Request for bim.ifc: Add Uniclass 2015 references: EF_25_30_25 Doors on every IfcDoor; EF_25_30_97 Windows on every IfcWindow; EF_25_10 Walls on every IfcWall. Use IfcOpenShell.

First a look at what the model holds.

```python
import ifcopenshell

model = ifcopenshell.open("bim.ifc")
print(model.schema)
print("classifications:", [c.Name for c in model.by_type("IfcClassification")])
for ifc_class in ("IfcDoor", "IfcRoof", "IfcStair", "IfcWall", "IfcWindow"):
    print(ifc_class, len(model.by_type(ifc_class)))
```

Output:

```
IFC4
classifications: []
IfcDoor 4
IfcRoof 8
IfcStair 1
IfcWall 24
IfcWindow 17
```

```python
import ifcopenshell
import ifcopenshell.api.classification

model = ifcopenshell.open("bim.ifc")

system = ifcopenshell.api.classification.add_classification(model, classification="Uniclass 2015")

codes = {
    "IfcDoor": ("EF_25_30_25", "Doors"),
    "IfcWindow": ("EF_25_30_97", "Windows"),
    "IfcWall": ("EF_25_10", "Walls"),
}
for ifc_class, (code, name) in codes.items():
    products = model.by_type(ifc_class)
    ifcopenshell.api.classification.add_reference(
        model, products=products, classification=system, identification=code, name=name
    )
    print(code, len(products))

model.write("bim_edited.ifc")
```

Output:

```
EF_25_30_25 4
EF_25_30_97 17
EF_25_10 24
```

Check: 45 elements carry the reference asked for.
